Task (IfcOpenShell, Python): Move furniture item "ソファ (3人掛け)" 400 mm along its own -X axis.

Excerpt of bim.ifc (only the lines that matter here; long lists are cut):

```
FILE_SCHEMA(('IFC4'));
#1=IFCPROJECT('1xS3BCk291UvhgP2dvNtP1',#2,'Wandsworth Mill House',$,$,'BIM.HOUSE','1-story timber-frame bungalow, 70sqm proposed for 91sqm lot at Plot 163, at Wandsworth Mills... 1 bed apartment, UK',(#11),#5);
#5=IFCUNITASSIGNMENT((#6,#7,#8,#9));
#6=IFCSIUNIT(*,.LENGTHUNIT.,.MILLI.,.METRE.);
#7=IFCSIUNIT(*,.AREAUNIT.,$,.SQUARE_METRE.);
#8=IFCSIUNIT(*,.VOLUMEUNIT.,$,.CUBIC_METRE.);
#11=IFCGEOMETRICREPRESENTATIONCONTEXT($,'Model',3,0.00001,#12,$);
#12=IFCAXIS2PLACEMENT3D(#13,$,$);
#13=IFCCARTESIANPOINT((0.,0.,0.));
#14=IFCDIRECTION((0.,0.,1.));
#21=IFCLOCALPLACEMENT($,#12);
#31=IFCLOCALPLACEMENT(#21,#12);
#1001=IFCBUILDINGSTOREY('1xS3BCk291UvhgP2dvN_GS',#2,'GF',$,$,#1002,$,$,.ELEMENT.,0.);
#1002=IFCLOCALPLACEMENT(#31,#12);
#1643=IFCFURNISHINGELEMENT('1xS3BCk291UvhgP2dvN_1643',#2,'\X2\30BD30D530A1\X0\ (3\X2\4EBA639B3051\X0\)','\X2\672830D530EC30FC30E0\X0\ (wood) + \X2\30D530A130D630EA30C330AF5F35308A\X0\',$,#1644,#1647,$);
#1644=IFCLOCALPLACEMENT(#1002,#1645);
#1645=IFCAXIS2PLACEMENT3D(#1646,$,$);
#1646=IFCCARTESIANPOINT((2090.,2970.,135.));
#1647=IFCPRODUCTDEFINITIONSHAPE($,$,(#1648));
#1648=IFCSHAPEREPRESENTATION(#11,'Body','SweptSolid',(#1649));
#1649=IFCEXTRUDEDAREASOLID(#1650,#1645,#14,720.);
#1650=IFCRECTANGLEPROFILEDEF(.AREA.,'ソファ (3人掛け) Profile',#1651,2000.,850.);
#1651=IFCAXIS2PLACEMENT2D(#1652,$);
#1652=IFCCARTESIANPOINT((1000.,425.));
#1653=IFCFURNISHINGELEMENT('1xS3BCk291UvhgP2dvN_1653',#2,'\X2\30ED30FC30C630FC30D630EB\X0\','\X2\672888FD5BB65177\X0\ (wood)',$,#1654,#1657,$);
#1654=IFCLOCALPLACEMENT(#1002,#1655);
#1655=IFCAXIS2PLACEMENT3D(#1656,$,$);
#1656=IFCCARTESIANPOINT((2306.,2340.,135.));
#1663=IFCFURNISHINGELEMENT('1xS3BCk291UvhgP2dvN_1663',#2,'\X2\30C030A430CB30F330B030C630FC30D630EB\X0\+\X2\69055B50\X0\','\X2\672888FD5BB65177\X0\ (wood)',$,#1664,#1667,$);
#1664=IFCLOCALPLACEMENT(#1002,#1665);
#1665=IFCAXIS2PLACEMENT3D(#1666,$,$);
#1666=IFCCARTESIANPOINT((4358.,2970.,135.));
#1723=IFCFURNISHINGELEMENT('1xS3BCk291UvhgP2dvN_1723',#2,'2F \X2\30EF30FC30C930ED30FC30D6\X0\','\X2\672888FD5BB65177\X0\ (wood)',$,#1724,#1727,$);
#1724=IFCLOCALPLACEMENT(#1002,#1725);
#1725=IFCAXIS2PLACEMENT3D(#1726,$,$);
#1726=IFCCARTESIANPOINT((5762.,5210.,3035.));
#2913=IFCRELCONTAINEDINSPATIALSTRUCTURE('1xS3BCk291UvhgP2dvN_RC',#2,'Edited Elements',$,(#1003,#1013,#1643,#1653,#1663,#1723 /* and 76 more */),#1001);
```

```python
import ifcopenshell
import ifcopenshell.api.geometry
import ifcopenshell.util.placement

model = ifcopenshell.open("bim.ifc")

item = model.by_id(1643)
matrix = ifcopenshell.util.placement.get_local_placement(item.ObjectPlacement)
matrix[:3, 3] -= matrix[:3, 0] * 400.0
ifcopenshell.api.geometry.edit_object_placement(model, product=item, matrix=matrix, is_si=False)

print(ifcopenshell.util.placement.get_local_placement(item.ObjectPlacement).round(3) + 0.0)

model.write("bim_edited.ifc")
```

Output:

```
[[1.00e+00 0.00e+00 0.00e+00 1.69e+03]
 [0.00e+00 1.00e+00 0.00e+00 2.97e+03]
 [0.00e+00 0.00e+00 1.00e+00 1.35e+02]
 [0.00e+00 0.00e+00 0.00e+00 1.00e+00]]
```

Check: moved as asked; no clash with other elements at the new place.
